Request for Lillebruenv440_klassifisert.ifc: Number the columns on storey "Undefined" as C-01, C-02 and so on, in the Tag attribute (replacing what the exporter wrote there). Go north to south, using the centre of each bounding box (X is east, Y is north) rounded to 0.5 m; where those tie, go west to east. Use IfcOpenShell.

First a look at what the model holds.

```python
import ifcopenshell
import ifcopenshell.util.element
import ifcopenshell.util.placement

model = ifcopenshell.open("Lillebruenv440_klassifisert.ifc")
print(model.schema)
storey = next(s for s in model.by_type("IfcBuildingStorey") if s.Name == "Undefined")
columns = [e for e in ifcopenshell.util.element.get_decomposition(storey) if e.is_a("IfcColumn")]
for e in sorted(columns, key=lambda e: e.id()):
    origin = ifcopenshell.util.placement.get_local_placement(e.ObjectPlacement)[:3, 3]
    print(e.id(), e.Tag, e.Name, origin.round(2) + 0.0, sep=" | ")
```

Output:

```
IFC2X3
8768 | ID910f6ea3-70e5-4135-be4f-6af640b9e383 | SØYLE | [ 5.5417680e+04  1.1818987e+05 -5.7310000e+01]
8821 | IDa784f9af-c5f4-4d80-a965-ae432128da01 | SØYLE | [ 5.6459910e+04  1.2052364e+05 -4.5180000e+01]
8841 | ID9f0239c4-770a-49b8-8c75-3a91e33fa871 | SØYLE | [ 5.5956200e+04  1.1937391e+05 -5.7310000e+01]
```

```python
import ifcopenshell
import ifcopenshell.geom
import ifcopenshell.util.element
import ifcopenshell.util.shape

model = ifcopenshell.open("Lillebruenv440_klassifisert.ifc")
settings = ifcopenshell.geom.settings()
settings.set("use-world-coords", True)


def centre(element):
    shape = ifcopenshell.geom.create_shape(settings, element)
    return ifcopenshell.util.shape.get_bbox_centroid(shape.geometry)


storey = next(s for s in model.by_type("IfcBuildingStorey") if s.Name == "Undefined")
columns = [e for e in ifcopenshell.util.element.get_decomposition(storey) if e.is_a("IfcColumn")]

# Insertion points can sit at a corner or the storey origin, so sort by the geometry (in metres).
centres = {e: centre(e) for e in columns}
columns.sort(key=lambda e: (-round(centres[e][1] / 0.5), centres[e][0]))

for i, e in enumerate(columns, start=1):
    number = f"C-{i:02d}"
    e.Tag = number
    print(e.id(), number)

model.write("Lillebruenv440_klassifisert_updated.ifc")
```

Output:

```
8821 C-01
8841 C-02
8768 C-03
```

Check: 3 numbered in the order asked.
